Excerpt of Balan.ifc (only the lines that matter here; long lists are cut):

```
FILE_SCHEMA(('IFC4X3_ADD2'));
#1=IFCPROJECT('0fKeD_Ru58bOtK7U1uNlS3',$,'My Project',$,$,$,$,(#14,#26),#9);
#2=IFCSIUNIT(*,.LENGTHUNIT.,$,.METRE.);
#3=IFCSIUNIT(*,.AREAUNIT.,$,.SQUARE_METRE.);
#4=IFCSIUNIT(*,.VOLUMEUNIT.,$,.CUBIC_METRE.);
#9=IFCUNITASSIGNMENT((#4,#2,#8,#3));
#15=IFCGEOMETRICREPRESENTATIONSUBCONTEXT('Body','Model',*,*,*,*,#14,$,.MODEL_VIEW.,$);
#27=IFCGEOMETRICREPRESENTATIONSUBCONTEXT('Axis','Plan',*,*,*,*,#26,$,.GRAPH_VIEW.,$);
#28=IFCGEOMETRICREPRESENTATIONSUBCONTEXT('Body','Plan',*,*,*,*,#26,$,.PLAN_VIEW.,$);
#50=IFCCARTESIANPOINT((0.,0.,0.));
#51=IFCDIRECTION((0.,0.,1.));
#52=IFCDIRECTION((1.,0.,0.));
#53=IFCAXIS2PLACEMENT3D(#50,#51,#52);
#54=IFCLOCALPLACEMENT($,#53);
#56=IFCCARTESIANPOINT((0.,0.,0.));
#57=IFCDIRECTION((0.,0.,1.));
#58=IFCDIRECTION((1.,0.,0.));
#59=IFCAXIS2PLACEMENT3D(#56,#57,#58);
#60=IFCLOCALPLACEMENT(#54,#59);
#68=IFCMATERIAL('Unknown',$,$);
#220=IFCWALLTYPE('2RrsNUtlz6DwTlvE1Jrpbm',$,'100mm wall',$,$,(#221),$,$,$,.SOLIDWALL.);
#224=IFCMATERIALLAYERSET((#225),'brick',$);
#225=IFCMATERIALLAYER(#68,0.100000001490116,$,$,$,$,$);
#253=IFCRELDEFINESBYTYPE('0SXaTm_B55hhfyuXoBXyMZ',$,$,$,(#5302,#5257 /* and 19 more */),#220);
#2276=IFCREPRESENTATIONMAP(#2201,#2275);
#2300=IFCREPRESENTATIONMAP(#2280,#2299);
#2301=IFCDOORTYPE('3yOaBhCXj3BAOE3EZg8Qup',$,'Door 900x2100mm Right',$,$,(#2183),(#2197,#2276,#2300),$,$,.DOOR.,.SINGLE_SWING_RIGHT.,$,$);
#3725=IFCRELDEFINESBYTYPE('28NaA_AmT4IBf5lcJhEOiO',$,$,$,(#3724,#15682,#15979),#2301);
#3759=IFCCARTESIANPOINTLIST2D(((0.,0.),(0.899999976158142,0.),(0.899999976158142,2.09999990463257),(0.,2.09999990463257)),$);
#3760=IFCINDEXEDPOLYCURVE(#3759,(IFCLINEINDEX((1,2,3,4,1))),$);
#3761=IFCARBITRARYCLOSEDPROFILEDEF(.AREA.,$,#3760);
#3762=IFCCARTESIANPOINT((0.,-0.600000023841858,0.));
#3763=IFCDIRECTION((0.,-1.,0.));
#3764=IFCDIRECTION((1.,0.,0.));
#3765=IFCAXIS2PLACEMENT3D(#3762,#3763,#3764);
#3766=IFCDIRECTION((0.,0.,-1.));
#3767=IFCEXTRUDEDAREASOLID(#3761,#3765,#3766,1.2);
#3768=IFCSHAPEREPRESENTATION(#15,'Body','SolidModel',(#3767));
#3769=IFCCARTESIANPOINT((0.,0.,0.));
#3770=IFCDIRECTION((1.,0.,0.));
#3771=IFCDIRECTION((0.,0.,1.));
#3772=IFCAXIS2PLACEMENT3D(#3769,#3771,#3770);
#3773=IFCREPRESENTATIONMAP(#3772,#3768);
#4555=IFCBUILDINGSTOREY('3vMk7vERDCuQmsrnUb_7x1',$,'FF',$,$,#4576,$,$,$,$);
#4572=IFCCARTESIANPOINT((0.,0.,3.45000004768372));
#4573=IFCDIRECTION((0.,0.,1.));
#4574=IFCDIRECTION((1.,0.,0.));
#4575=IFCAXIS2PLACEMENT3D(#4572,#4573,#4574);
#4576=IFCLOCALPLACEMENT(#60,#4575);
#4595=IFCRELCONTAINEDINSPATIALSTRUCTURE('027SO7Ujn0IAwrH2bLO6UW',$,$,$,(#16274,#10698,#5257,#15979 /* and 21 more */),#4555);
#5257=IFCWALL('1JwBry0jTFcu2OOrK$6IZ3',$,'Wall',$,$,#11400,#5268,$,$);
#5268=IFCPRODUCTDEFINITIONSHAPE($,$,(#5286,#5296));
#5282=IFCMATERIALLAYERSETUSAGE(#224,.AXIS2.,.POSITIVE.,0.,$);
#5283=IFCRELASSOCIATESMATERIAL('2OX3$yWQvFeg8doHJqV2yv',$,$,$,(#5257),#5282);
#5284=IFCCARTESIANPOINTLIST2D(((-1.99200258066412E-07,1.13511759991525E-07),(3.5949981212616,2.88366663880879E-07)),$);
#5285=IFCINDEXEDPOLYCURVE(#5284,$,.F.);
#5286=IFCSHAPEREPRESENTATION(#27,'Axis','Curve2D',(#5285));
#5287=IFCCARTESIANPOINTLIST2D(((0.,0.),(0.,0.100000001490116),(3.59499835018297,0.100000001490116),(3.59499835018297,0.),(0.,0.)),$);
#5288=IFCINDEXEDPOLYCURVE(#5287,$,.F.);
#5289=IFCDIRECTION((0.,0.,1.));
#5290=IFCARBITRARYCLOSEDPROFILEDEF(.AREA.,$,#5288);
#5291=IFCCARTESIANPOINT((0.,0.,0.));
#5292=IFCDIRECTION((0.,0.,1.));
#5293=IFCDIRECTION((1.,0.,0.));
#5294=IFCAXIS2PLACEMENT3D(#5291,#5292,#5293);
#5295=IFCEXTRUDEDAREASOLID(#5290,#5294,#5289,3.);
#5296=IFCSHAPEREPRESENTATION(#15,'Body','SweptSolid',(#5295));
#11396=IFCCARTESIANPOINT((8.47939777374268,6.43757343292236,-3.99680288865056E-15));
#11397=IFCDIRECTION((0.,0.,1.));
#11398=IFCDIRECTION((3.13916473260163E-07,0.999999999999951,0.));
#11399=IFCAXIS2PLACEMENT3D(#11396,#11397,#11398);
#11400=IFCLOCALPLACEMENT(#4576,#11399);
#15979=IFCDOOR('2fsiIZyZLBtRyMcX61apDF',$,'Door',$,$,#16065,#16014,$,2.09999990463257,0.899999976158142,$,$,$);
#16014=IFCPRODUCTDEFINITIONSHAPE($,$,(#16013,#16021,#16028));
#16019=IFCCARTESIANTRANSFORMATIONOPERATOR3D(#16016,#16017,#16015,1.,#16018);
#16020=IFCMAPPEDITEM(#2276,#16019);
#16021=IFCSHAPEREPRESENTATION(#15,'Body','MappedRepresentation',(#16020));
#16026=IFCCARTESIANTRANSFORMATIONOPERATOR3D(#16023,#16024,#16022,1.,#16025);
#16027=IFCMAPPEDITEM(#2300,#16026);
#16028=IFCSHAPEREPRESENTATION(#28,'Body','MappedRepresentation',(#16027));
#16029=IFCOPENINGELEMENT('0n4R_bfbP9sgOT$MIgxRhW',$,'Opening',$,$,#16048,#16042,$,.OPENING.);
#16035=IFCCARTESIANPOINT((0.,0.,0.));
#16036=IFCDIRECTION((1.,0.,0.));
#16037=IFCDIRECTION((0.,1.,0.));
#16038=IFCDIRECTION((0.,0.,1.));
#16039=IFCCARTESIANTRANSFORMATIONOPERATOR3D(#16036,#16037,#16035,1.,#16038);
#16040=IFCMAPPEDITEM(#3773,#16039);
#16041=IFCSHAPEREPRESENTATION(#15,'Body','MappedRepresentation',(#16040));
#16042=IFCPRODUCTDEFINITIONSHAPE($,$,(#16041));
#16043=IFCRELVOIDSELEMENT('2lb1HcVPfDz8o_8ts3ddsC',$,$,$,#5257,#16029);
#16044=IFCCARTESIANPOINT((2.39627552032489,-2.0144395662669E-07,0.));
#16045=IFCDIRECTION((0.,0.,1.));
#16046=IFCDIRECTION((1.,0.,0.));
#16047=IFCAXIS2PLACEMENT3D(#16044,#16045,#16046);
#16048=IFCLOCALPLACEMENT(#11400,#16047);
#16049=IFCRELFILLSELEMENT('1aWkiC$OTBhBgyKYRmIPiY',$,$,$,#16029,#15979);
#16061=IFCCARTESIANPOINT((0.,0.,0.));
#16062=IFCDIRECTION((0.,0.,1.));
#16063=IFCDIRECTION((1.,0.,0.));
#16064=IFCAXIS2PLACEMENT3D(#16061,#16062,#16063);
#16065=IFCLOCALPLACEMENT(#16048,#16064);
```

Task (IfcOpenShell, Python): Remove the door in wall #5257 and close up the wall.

```python
import ifcopenshell
import ifcopenshell.api.feature
import ifcopenshell.api.root
import ifcopenshell.geom
import ifcopenshell.util.shape

model = ifcopenshell.open("Balan.ifc")
settings = ifcopenshell.geom.settings()


def volume(element):
    """Net volume in cubic metres, openings subtracted."""
    shape = ifcopenshell.geom.create_shape(settings, element)
    return ifcopenshell.util.shape.get_volume(shape.geometry)


door = model.by_id(15979)
opening = door.FillsVoids[0].RelatingOpeningElement
wall = opening.VoidsElements[0].RelatingBuildingElement
before = volume(wall)

ifcopenshell.api.root.remove_product(model, product=door)
ifcopenshell.api.feature.remove_feature(model, feature=opening)

after = volume(wall)

print(f"wall volume {before:.3f} -> {after:.3f} m3")

model.write("Balan_v2.ifc")
```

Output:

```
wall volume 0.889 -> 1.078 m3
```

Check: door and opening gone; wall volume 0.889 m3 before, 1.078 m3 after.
